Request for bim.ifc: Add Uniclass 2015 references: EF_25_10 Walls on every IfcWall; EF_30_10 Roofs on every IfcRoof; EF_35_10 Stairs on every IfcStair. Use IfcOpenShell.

First a look at what the model holds.

```python
import ifcopenshell

model = ifcopenshell.open("bim.ifc")
print(model.schema)
print("classifications:", [c.Name for c in model.by_type("IfcClassification")])
for ifc_class in ("IfcDoor", "IfcRoof", "IfcStair", "IfcWall", "IfcWindow"):
    print(ifc_class, len(model.by_type(ifc_class)))
```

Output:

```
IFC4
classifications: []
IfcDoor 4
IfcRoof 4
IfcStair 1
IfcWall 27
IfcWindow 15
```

```python
import ifcopenshell
import ifcopenshell.api.classification

model = ifcopenshell.open("bim.ifc")

system = ifcopenshell.api.classification.add_classification(model, classification="Uniclass 2015")

codes = {
    "IfcWall": ("EF_25_10", "Walls"),
    "IfcRoof": ("EF_30_10", "Roofs"),
    "IfcStair": ("EF_35_10", "Stairs"),
}
for ifc_class, (code, name) in codes.items():
    products = model.by_type(ifc_class)
    ifcopenshell.api.classification.add_reference(
        model, products=products, classification=system, identification=code, name=name
    )
    print(code, len(products))

model.write("bim_v2.ifc")
```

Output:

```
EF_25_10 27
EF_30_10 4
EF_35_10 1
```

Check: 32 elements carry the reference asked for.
